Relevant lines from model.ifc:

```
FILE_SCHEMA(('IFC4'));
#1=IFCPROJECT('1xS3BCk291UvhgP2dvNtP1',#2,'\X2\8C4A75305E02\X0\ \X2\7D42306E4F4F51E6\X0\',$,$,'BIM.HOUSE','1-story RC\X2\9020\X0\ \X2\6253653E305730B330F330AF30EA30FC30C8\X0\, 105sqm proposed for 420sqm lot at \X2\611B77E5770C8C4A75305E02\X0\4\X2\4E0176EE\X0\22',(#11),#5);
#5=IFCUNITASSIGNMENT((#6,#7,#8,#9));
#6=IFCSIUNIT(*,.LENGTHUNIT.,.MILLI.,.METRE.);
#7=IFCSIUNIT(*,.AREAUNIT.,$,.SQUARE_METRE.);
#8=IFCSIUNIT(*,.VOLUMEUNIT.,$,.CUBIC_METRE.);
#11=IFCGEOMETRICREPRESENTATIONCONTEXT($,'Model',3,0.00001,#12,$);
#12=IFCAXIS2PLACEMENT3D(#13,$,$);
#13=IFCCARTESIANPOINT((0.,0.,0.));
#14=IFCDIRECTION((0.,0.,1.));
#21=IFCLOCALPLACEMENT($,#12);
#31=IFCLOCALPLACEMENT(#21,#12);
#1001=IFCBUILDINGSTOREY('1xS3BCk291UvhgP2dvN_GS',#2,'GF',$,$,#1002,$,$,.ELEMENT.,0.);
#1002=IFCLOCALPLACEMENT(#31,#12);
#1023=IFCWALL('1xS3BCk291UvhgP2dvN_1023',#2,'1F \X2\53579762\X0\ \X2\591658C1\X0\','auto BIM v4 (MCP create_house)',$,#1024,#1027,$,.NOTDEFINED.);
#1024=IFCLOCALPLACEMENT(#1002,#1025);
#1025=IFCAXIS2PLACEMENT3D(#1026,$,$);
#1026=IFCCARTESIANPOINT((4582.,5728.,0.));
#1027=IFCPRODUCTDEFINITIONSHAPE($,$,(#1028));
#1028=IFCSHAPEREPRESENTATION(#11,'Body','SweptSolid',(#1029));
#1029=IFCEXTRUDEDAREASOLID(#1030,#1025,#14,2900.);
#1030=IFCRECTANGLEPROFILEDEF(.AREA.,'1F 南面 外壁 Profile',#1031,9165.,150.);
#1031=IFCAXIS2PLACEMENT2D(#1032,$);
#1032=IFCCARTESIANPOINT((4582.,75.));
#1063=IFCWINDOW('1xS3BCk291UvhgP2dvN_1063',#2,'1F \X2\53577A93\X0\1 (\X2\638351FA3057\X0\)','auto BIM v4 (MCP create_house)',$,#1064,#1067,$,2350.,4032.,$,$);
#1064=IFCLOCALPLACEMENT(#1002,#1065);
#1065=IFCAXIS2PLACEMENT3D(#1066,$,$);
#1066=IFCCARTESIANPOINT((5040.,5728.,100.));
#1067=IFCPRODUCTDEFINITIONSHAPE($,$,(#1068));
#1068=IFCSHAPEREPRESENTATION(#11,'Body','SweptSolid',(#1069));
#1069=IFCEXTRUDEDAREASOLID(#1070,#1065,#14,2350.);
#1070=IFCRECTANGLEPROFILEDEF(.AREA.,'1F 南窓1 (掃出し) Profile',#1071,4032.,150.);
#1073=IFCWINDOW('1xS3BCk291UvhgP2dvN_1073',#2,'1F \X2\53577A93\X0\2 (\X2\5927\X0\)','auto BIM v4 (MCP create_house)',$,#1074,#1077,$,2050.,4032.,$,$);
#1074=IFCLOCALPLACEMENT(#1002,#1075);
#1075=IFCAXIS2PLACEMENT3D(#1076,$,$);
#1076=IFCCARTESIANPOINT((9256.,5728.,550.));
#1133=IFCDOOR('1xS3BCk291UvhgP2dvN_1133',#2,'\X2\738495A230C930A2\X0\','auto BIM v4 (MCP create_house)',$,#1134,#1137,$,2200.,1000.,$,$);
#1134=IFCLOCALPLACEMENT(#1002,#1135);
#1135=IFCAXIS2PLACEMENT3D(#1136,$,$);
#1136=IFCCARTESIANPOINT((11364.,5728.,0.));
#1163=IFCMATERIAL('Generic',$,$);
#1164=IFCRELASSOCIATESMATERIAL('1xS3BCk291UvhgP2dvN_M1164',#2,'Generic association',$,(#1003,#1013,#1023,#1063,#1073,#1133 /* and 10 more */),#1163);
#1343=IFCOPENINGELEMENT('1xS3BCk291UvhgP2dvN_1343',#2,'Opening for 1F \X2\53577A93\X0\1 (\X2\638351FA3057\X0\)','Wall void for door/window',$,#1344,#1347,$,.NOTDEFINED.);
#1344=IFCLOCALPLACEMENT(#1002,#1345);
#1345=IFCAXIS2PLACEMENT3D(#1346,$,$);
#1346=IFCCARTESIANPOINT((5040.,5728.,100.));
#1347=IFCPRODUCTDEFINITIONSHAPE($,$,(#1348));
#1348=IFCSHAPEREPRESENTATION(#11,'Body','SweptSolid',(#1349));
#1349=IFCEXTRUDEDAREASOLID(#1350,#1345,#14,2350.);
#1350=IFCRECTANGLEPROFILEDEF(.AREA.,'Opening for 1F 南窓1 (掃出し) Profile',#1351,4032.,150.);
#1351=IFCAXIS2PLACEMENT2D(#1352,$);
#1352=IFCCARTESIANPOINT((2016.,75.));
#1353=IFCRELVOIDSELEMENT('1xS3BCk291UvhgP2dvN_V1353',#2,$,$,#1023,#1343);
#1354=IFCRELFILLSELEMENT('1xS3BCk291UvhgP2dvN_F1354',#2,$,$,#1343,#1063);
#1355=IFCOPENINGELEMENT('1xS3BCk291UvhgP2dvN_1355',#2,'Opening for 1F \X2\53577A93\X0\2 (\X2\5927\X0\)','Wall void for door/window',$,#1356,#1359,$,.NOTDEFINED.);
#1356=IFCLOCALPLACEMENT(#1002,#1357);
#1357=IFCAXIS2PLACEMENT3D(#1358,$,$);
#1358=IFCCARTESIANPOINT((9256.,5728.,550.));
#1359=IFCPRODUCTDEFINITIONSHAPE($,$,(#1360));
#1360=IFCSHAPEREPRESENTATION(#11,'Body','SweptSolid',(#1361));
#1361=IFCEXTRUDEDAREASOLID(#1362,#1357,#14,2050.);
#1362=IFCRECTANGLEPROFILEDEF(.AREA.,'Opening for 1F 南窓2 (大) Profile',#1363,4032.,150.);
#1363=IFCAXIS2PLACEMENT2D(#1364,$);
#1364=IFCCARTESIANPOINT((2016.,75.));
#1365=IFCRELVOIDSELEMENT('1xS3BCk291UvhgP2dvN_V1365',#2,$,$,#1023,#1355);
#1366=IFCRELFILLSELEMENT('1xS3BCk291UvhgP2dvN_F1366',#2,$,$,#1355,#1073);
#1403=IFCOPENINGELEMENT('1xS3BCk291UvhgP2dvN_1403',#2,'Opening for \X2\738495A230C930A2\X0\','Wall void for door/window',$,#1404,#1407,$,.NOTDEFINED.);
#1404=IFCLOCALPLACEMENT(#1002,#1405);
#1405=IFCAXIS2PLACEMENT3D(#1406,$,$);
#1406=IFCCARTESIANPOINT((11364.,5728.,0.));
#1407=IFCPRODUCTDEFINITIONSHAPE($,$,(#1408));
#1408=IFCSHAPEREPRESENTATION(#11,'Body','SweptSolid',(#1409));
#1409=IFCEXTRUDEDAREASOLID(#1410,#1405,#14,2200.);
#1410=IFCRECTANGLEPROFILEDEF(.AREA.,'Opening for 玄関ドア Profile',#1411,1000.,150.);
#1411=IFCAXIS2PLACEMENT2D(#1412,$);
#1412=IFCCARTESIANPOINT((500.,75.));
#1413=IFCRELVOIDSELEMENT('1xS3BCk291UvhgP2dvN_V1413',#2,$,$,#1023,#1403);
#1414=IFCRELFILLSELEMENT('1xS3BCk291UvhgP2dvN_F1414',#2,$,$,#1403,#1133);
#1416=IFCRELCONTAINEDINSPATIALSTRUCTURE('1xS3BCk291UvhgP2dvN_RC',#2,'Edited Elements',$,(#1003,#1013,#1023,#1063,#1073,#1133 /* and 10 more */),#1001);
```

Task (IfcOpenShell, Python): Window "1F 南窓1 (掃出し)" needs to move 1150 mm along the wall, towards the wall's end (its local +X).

```python
import ifcopenshell
import ifcopenshell.api.geometry
import ifcopenshell.util.placement
import ifcopenshell.util.unit

model = ifcopenshell.open("model.ifc")
unit_scale = ifcopenshell.util.unit.calculate_unit_scale(model)

window = model.by_guid("1xS3BCk291UvhgP2dvN_1063")
opening = window.FillsVoids[0].RelatingOpeningElement
wall = opening.VoidsElements[0].RelatingBuildingElement

wall_matrix = ifcopenshell.util.placement.get_local_placement(wall.ObjectPlacement)
shift = wall_matrix[:3, 0] * 1.15 / unit_scale
before = ifcopenshell.util.placement.get_local_placement(window.ObjectPlacement)[:3, 3].copy()

# The window is not placed relative to its opening, so move both.
for product in (opening, window):
    matrix = ifcopenshell.util.placement.get_local_placement(product.ObjectPlacement)
    matrix[:3, 3] += shift
    ifcopenshell.api.geometry.edit_object_placement(model, product=product, matrix=matrix, is_si=False)

after = ifcopenshell.util.placement.get_local_placement(window.ObjectPlacement)[:3, 3]
print("window moved by", (after - before).round(3) + 0.0)

model.write("model_v2.ifc")
```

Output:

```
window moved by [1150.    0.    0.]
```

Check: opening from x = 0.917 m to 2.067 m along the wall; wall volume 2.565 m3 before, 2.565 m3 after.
